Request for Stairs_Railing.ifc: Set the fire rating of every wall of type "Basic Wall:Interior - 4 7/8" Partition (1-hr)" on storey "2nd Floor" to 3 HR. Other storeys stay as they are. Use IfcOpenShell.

First a look at what the model holds.

```python
import ifcopenshell
import ifcopenshell.util.element

model = ifcopenshell.open("Stairs_Railing.ifc")
print(model.schema)
storey = next(s for s in model.by_type("IfcBuildingStorey") if s.Name == "2nd Floor")
walls = [e for e in ifcopenshell.util.element.get_decomposition(storey) if e.is_a("IfcWall")]
seen = {}
for e in walls:
    element_type = ifcopenshell.util.element.get_type(e)
    key = (element_type.Name if element_type != e and element_type else None, ifcopenshell.util.element.get_pset(e, "Pset_WallCommon", "FireRating"))
    seen[key] = seen.get(key, 0) + 1
for (name, value), count in sorted(seen.items(), key=str):
    print(count, "x", name, "|", value)
```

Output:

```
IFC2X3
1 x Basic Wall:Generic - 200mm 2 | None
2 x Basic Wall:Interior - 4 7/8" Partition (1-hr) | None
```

```python
import ifcopenshell
import ifcopenshell.api.pset
import ifcopenshell.util.element

model = ifcopenshell.open("Stairs_Railing.ifc")

storey = next(s for s in model.by_type("IfcBuildingStorey") if s.Name == "2nd Floor")
walls = [e for e in ifcopenshell.util.element.get_decomposition(storey) if e.is_a("IfcWall")]

count = 0
for e in walls:
    element_type = ifcopenshell.util.element.get_type(e)
    if element_type in (None, e) or element_type.Name != 'Basic Wall:Interior - 4 7/8" Partition (1-hr)':
        continue
    # add_pset returns the element's existing set when there is one.
    pset = ifcopenshell.api.pset.add_pset(model, product=e, name="Pset_WallCommon")
    ifcopenshell.api.pset.edit_pset(model, pset=pset, properties={"FireRating": "3 HR"})
    count += 1

print(count, "walls updated")

model.write("Stairs_Railing-out.ifc")
```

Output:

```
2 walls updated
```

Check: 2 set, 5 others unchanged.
